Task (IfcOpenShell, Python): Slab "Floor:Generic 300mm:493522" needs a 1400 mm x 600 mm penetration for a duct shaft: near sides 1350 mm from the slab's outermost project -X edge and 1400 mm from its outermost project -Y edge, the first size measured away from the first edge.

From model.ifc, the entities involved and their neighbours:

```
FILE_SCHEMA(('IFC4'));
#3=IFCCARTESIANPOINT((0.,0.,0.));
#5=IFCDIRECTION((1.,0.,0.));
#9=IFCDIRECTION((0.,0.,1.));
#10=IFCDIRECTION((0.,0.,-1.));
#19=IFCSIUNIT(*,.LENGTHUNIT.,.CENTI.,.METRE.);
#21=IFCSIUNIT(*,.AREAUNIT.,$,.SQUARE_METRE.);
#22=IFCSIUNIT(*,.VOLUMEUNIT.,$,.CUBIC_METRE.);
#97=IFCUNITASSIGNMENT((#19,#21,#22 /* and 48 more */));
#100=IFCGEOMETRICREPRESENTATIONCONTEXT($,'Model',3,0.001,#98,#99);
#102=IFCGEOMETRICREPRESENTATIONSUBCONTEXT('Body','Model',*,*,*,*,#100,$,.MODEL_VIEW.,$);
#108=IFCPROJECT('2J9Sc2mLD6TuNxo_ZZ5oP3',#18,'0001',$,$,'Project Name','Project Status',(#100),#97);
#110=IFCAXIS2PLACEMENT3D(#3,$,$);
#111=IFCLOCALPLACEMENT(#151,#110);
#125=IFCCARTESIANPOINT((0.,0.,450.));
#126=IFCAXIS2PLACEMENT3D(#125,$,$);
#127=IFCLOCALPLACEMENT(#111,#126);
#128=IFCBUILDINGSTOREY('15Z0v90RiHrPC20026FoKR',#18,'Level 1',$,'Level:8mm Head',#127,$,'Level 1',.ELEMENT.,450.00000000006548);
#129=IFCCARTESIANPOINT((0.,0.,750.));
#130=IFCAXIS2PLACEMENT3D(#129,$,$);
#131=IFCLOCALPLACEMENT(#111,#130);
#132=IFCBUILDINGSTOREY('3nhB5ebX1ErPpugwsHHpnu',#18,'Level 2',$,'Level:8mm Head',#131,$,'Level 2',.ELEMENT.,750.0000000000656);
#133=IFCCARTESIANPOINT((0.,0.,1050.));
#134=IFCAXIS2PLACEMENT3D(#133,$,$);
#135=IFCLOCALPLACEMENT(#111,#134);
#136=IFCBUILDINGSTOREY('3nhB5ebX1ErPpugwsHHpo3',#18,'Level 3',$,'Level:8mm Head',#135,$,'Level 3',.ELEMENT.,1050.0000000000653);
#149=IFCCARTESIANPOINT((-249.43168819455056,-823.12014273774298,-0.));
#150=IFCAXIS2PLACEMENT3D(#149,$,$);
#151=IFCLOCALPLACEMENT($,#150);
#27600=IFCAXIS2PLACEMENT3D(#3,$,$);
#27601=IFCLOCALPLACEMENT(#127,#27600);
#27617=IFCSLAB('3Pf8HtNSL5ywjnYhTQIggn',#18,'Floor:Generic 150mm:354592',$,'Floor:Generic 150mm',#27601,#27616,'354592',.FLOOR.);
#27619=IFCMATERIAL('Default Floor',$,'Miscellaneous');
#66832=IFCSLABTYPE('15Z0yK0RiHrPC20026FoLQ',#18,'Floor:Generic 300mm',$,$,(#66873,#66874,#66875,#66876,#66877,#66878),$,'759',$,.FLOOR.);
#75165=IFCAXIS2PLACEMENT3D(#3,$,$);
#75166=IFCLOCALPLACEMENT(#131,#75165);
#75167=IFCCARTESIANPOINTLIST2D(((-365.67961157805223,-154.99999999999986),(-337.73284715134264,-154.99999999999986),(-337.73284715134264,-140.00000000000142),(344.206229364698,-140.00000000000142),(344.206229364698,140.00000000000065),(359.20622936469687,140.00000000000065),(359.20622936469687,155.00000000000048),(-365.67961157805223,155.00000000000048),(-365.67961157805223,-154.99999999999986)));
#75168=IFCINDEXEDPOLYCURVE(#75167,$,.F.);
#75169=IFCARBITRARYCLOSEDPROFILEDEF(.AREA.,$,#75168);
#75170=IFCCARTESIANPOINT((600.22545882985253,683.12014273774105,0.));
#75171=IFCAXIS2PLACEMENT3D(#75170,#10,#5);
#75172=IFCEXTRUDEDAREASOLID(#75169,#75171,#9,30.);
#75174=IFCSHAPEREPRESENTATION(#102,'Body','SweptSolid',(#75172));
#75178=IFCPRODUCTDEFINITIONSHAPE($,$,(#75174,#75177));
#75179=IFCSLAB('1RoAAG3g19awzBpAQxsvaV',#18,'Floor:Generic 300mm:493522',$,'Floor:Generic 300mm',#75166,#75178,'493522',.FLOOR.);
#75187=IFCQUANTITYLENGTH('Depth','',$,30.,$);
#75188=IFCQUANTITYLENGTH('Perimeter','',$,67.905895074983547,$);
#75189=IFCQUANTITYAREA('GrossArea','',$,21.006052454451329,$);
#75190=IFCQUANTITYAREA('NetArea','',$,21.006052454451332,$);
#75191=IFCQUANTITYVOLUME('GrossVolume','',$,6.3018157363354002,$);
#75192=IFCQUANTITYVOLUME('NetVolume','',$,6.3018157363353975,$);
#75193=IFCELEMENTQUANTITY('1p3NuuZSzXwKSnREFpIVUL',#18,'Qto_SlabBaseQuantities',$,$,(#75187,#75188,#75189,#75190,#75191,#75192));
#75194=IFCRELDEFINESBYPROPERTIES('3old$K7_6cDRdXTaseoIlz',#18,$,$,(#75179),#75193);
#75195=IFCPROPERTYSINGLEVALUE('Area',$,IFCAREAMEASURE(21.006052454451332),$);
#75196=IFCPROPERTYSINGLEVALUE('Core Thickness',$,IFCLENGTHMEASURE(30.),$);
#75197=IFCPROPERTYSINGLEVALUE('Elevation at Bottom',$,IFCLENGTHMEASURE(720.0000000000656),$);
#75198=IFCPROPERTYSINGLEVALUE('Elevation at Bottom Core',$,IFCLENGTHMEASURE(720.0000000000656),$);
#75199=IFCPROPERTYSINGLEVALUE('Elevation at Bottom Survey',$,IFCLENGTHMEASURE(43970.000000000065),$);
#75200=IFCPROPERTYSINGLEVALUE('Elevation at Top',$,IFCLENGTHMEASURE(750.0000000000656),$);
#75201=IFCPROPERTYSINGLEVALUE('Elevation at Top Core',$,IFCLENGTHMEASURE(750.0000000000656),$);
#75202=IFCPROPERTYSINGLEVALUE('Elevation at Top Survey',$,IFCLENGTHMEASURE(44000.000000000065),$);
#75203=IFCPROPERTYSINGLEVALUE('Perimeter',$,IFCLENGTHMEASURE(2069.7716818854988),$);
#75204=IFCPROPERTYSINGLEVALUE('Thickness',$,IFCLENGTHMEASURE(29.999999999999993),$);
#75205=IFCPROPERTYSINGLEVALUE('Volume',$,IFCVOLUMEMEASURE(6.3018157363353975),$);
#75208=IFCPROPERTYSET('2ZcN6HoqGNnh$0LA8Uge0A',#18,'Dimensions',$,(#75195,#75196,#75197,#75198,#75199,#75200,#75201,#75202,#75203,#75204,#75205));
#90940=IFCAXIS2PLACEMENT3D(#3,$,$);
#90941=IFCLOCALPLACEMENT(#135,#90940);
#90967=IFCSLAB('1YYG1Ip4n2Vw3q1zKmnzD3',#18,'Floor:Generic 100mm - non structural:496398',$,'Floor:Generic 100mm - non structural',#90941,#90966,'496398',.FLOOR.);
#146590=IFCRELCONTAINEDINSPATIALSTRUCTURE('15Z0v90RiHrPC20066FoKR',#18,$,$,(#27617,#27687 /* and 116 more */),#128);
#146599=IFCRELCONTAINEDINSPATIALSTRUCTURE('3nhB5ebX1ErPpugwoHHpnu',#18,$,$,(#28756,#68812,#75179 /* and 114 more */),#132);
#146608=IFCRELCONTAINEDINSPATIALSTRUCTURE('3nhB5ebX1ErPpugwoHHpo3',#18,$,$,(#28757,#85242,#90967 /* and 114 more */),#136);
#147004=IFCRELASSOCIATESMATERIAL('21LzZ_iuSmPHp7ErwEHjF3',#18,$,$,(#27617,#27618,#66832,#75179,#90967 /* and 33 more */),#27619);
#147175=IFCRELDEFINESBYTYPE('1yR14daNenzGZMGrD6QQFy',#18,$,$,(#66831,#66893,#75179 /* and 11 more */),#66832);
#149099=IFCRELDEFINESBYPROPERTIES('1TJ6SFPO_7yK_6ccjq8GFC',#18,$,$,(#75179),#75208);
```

```python
import numpy as np
import ifcopenshell
import ifcopenshell.api.feature
import ifcopenshell.api.geometry
import ifcopenshell.api.pset
import ifcopenshell.api.root
import ifcopenshell.geom
import ifcopenshell.util.element
import ifcopenshell.util.placement
import ifcopenshell.util.representation
import ifcopenshell.util.shape
import ifcopenshell.util.unit

model = ifcopenshell.open("model.ifc")
unit_scale = ifcopenshell.util.unit.calculate_unit_scale(model)
area_scale = ifcopenshell.util.unit.calculate_unit_scale(model, "AREAUNIT")
volume_scale = ifcopenshell.util.unit.calculate_unit_scale(model, "VOLUMEUNIT")
settings = ifcopenshell.geom.settings()


def volume(element):
    """Net volume in cubic metres, openings subtracted."""
    shape = ifcopenshell.geom.create_shape(settings, element)
    return ifcopenshell.util.shape.get_volume(shape.geometry)


slab = model.by_id(75179)
before = volume(slab)

# Extent in the slab's own axes, in metres. The edges named are its -X and -Y sides.
slab_shape = ifcopenshell.geom.create_shape(settings, slab)
vertices = ifcopenshell.util.shape.get_vertices(slab_shape.geometry)
x_min, y_min, bottom = vertices.min(axis=0)
top = vertices[:, 2].max()

opening = ifcopenshell.api.root.create_entity(model, ifc_class="IfcOpeningElement", name="Duct shaft opening", predefined_type="OPENING")
context = ifcopenshell.util.representation.get_context(model, "Model", "Body", "MODEL_VIEW")
width, depth = 1.4, 0.6
outline = [(0.0, 0.0), (width, 0.0), (width, depth), (0.0, depth), (0.0, 0.0)]
# Overshoot both faces by 50 mm so the cut is clean.
shape = ifcopenshell.api.geometry.add_slab_representation(
    model, context=context, depth=top - bottom + 0.1, polyline=outline
)
ifcopenshell.api.geometry.assign_representation(model, product=opening, representation=shape)

matrix = ifcopenshell.util.placement.get_local_placement(slab.ObjectPlacement)
matrix[:, 3] = matrix @ np.append(np.array([x_min + 1.35, y_min + 1.4, bottom - 0.05]) / unit_scale, 1.0)
ifcopenshell.api.geometry.edit_object_placement(model, product=opening, matrix=matrix, is_si=False)
ifcopenshell.api.feature.add_feature(model, feature=opening, element=slab)

after = volume(slab)

# Update the slab's stored quantities.
qto = model.by_id(ifcopenshell.util.element.get_pset(slab, "Qto_SlabBaseQuantities", should_inherit=False)["id"])
ifcopenshell.api.pset.edit_qto(model, qto=qto, properties={
    "NetArea": after / (top - bottom) / area_scale,
    "NetVolume": after / volume_scale,
})
pset = model.by_id(ifcopenshell.util.element.get_pset(slab, "Dimensions", should_inherit=False)["id"])
ifcopenshell.api.pset.edit_pset(model, pset=pset, properties={
    "Area": model.create_entity("IfcAreaMeasure", after / (top - bottom) / area_scale),
    "Volume": model.create_entity("IfcVolumeMeasure", after / volume_scale),
})

print(f"slab volume {before:.3f} -> {after:.3f} m3")

model.write("model_v2.ifc")
```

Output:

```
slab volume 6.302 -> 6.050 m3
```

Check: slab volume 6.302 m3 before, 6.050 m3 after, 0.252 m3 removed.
